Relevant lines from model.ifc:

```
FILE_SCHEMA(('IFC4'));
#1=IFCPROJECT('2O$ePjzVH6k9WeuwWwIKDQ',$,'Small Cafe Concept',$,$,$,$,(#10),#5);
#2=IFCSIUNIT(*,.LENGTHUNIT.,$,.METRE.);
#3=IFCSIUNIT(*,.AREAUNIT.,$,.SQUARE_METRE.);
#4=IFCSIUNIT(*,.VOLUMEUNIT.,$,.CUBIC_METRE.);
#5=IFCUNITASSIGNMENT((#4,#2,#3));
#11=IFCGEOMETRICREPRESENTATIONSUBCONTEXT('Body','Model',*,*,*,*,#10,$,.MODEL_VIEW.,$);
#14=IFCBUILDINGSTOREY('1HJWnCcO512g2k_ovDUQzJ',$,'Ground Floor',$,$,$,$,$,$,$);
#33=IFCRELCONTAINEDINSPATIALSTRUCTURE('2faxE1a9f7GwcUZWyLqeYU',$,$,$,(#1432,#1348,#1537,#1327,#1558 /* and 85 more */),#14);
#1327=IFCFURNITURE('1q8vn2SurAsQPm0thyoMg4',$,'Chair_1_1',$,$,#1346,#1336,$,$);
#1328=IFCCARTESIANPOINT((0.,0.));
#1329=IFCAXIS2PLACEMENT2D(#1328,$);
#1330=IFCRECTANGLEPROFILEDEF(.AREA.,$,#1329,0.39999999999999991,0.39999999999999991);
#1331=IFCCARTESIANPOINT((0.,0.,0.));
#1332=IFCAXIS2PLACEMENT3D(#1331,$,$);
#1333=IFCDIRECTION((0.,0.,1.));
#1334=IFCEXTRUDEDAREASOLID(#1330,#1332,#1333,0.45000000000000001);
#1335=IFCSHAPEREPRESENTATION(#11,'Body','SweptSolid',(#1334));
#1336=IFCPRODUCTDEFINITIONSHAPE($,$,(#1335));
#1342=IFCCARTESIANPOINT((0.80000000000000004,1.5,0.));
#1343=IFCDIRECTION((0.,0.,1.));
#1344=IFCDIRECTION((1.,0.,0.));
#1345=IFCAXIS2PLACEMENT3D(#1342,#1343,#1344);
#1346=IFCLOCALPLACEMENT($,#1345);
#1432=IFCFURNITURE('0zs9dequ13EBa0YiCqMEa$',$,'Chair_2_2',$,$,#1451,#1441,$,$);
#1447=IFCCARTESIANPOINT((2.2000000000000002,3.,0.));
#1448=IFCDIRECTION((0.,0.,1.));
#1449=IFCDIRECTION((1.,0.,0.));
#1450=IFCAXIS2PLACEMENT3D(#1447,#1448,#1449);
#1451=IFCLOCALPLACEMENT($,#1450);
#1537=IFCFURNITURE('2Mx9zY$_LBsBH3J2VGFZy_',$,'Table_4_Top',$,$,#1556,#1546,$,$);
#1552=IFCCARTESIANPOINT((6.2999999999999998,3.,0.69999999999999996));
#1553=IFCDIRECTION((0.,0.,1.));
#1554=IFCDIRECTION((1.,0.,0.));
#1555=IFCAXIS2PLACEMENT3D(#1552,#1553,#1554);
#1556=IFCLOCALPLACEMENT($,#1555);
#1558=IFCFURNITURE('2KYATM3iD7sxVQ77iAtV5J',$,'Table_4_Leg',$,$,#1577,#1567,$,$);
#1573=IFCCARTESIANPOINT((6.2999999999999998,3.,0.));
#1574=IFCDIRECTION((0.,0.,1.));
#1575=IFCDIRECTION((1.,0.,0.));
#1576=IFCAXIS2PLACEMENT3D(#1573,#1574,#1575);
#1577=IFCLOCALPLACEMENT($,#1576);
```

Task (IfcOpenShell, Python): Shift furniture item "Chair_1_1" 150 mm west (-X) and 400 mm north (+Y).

```python
import ifcopenshell
import ifcopenshell.api.geometry
import ifcopenshell.util.placement
import ifcopenshell.util.unit

model = ifcopenshell.open("model.ifc")
unit_scale = ifcopenshell.util.unit.calculate_unit_scale(model)

item = model.by_guid("1q8vn2SurAsQPm0thyoMg4")
matrix = ifcopenshell.util.placement.get_local_placement(item.ObjectPlacement)
matrix[0, 3] -= 0.15 / unit_scale
matrix[1, 3] += 0.4 / unit_scale
ifcopenshell.api.geometry.edit_object_placement(model, product=item, matrix=matrix, is_si=False)

print(ifcopenshell.util.placement.get_local_placement(item.ObjectPlacement).round(3) + 0.0)

model.write("model_edited.ifc")
```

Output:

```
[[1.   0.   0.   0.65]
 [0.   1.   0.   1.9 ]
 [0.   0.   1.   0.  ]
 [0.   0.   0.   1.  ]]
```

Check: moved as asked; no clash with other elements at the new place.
